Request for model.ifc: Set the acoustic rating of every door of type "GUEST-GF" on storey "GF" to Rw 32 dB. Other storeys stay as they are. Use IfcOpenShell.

First a look at what the model holds.

```python
import ifcopenshell
import ifcopenshell.util.element

model = ifcopenshell.open("model.ifc")
print(model.schema)
storey = next(s for s in model.by_type("IfcBuildingStorey") if s.Name == "GF")
doors = [e for e in ifcopenshell.util.element.get_decomposition(storey) if e.is_a("IfcDoor")]
seen = {}
for e in doors:
    element_type = ifcopenshell.util.element.get_type(e)
    key = (element_type.Name if element_type != e and element_type else None, ifcopenshell.util.element.get_pset(e, "Pset_DoorCommon", "AcousticRating"))
    seen[key] = seen.get(key, 0) + 1
for (name, value), count in sorted(seen.items(), key=str):
    print(count, "x", name, "|", value)
```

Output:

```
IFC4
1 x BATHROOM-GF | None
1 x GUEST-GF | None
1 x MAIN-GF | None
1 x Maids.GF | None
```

```python
import ifcopenshell
import ifcopenshell.api.pset
import ifcopenshell.util.element

model = ifcopenshell.open("model.ifc")

storey = next(s for s in model.by_type("IfcBuildingStorey") if s.Name == "GF")
doors = [e for e in ifcopenshell.util.element.get_decomposition(storey) if e.is_a("IfcDoor")]

count = 0
for e in doors:
    element_type = ifcopenshell.util.element.get_type(e)
    if element_type in (None, e) or element_type.Name != "GUEST-GF":
        continue
    # add_pset returns the element's existing set when there is one.
    pset = ifcopenshell.api.pset.add_pset(model, product=e, name="Pset_DoorCommon")
    ifcopenshell.api.pset.edit_pset(model, pset=pset, properties={"AcousticRating": "Rw 32 dB"})
    count += 1

print(count, "doors updated")

model.write("model_edited.ifc")
```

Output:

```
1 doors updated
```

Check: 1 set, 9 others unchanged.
